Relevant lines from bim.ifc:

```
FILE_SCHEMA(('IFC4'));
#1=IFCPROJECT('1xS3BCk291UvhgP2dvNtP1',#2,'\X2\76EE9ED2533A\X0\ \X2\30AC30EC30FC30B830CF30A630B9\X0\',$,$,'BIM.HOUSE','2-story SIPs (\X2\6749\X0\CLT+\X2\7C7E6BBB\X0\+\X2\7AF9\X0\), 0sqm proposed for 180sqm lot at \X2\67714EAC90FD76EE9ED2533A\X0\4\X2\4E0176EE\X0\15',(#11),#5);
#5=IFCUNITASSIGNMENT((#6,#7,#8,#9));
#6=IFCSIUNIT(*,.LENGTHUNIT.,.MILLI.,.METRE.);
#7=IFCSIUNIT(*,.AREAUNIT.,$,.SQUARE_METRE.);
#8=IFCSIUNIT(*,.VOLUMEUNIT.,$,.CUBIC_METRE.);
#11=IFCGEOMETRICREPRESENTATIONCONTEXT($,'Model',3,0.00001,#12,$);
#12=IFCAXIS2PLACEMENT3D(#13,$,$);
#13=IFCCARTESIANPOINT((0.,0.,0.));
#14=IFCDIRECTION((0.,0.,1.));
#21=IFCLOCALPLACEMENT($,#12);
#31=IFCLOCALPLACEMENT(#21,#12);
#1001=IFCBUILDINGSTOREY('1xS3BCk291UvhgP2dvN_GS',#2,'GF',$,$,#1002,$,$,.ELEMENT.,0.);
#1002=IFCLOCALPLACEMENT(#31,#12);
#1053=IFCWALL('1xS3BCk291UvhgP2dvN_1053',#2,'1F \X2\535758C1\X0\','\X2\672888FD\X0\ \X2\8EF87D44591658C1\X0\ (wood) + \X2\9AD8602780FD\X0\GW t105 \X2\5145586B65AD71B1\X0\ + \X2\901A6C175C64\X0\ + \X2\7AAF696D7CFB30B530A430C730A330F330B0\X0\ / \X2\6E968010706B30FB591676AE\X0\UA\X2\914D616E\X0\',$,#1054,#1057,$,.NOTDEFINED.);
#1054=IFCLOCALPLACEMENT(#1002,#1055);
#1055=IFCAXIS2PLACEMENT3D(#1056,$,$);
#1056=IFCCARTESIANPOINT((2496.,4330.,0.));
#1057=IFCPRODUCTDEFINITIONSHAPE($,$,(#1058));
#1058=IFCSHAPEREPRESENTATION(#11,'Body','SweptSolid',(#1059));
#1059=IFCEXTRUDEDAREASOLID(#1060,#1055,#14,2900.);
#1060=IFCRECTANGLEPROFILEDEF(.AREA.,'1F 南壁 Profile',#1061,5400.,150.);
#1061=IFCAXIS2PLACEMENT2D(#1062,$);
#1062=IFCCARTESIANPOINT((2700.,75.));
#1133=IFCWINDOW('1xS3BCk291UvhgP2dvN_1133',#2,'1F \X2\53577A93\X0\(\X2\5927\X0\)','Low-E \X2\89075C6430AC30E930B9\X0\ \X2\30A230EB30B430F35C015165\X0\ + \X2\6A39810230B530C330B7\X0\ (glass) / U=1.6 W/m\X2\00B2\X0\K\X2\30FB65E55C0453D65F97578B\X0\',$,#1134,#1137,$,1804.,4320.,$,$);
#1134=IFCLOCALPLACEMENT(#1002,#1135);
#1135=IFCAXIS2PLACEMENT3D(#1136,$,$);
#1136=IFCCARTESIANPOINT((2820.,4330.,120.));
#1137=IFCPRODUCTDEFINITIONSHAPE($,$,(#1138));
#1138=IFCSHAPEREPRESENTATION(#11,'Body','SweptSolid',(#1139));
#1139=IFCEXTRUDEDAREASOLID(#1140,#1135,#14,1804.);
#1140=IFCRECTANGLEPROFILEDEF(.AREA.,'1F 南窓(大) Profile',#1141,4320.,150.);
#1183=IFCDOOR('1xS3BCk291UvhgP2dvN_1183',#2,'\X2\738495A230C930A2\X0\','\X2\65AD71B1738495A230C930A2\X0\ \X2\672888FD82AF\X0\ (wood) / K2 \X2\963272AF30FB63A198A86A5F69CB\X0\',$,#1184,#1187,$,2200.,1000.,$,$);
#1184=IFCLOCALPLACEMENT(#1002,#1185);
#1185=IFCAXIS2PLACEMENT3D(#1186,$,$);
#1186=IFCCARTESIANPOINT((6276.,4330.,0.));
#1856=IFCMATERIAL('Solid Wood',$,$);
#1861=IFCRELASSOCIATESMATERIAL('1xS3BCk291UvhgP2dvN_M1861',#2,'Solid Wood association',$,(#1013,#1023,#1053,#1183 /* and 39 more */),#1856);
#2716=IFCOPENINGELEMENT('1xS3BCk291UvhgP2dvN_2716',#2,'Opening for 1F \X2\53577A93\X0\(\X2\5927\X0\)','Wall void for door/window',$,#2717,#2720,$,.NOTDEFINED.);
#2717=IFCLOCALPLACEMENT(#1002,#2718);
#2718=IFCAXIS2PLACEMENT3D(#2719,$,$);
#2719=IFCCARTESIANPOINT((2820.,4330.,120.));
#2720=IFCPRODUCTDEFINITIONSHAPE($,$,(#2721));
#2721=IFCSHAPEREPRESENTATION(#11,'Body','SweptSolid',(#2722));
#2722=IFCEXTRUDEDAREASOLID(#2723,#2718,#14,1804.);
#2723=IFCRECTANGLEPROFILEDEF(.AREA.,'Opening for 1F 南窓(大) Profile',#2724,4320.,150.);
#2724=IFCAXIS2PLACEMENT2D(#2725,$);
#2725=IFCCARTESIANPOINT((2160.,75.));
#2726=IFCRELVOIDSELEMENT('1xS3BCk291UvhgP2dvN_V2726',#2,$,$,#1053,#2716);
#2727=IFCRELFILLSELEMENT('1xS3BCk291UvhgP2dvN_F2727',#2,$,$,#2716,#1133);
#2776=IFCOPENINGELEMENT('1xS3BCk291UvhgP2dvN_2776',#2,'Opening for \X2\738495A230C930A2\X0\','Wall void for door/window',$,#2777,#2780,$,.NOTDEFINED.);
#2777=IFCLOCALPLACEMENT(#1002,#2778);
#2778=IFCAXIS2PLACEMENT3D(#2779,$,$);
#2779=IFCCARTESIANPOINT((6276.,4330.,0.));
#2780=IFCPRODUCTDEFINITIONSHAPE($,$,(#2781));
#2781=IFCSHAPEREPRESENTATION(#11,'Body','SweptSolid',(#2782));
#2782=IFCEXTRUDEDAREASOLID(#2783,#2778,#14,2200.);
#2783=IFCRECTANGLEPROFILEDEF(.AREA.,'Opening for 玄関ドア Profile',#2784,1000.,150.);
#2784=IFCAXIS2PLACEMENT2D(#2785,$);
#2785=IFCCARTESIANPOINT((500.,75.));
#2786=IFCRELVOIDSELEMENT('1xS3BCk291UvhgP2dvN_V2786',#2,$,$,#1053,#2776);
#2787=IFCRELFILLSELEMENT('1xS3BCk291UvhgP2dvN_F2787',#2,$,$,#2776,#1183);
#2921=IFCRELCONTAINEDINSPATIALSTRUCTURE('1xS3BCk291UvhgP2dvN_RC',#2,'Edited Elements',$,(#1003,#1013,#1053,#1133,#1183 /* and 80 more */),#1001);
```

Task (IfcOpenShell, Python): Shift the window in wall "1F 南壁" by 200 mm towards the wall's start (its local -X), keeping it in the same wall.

```python
import ifcopenshell
import ifcopenshell.api.geometry
import ifcopenshell.util.placement

model = ifcopenshell.open("bim.ifc")

window = model.by_guid("1xS3BCk291UvhgP2dvN_1133")
opening = window.FillsVoids[0].RelatingOpeningElement
wall = opening.VoidsElements[0].RelatingBuildingElement

wall_matrix = ifcopenshell.util.placement.get_local_placement(wall.ObjectPlacement)
shift = wall_matrix[:3, 0] * -200.0
before = ifcopenshell.util.placement.get_local_placement(window.ObjectPlacement)[:3, 3].copy()

# The window is not placed relative to its opening, so move both.
for product in (opening, window):
    matrix = ifcopenshell.util.placement.get_local_placement(product.ObjectPlacement)
    matrix[:3, 3] += shift
    ifcopenshell.api.geometry.edit_object_placement(model, product=product, matrix=matrix, is_si=False)

after = ifcopenshell.util.placement.get_local_placement(window.ObjectPlacement)[:3, 3]
print("window moved by", (after - before).round(3) + 0.0)

model.write("bim_edited.ifc")
```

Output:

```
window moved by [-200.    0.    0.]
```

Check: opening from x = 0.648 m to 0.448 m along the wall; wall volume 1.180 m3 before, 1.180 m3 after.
